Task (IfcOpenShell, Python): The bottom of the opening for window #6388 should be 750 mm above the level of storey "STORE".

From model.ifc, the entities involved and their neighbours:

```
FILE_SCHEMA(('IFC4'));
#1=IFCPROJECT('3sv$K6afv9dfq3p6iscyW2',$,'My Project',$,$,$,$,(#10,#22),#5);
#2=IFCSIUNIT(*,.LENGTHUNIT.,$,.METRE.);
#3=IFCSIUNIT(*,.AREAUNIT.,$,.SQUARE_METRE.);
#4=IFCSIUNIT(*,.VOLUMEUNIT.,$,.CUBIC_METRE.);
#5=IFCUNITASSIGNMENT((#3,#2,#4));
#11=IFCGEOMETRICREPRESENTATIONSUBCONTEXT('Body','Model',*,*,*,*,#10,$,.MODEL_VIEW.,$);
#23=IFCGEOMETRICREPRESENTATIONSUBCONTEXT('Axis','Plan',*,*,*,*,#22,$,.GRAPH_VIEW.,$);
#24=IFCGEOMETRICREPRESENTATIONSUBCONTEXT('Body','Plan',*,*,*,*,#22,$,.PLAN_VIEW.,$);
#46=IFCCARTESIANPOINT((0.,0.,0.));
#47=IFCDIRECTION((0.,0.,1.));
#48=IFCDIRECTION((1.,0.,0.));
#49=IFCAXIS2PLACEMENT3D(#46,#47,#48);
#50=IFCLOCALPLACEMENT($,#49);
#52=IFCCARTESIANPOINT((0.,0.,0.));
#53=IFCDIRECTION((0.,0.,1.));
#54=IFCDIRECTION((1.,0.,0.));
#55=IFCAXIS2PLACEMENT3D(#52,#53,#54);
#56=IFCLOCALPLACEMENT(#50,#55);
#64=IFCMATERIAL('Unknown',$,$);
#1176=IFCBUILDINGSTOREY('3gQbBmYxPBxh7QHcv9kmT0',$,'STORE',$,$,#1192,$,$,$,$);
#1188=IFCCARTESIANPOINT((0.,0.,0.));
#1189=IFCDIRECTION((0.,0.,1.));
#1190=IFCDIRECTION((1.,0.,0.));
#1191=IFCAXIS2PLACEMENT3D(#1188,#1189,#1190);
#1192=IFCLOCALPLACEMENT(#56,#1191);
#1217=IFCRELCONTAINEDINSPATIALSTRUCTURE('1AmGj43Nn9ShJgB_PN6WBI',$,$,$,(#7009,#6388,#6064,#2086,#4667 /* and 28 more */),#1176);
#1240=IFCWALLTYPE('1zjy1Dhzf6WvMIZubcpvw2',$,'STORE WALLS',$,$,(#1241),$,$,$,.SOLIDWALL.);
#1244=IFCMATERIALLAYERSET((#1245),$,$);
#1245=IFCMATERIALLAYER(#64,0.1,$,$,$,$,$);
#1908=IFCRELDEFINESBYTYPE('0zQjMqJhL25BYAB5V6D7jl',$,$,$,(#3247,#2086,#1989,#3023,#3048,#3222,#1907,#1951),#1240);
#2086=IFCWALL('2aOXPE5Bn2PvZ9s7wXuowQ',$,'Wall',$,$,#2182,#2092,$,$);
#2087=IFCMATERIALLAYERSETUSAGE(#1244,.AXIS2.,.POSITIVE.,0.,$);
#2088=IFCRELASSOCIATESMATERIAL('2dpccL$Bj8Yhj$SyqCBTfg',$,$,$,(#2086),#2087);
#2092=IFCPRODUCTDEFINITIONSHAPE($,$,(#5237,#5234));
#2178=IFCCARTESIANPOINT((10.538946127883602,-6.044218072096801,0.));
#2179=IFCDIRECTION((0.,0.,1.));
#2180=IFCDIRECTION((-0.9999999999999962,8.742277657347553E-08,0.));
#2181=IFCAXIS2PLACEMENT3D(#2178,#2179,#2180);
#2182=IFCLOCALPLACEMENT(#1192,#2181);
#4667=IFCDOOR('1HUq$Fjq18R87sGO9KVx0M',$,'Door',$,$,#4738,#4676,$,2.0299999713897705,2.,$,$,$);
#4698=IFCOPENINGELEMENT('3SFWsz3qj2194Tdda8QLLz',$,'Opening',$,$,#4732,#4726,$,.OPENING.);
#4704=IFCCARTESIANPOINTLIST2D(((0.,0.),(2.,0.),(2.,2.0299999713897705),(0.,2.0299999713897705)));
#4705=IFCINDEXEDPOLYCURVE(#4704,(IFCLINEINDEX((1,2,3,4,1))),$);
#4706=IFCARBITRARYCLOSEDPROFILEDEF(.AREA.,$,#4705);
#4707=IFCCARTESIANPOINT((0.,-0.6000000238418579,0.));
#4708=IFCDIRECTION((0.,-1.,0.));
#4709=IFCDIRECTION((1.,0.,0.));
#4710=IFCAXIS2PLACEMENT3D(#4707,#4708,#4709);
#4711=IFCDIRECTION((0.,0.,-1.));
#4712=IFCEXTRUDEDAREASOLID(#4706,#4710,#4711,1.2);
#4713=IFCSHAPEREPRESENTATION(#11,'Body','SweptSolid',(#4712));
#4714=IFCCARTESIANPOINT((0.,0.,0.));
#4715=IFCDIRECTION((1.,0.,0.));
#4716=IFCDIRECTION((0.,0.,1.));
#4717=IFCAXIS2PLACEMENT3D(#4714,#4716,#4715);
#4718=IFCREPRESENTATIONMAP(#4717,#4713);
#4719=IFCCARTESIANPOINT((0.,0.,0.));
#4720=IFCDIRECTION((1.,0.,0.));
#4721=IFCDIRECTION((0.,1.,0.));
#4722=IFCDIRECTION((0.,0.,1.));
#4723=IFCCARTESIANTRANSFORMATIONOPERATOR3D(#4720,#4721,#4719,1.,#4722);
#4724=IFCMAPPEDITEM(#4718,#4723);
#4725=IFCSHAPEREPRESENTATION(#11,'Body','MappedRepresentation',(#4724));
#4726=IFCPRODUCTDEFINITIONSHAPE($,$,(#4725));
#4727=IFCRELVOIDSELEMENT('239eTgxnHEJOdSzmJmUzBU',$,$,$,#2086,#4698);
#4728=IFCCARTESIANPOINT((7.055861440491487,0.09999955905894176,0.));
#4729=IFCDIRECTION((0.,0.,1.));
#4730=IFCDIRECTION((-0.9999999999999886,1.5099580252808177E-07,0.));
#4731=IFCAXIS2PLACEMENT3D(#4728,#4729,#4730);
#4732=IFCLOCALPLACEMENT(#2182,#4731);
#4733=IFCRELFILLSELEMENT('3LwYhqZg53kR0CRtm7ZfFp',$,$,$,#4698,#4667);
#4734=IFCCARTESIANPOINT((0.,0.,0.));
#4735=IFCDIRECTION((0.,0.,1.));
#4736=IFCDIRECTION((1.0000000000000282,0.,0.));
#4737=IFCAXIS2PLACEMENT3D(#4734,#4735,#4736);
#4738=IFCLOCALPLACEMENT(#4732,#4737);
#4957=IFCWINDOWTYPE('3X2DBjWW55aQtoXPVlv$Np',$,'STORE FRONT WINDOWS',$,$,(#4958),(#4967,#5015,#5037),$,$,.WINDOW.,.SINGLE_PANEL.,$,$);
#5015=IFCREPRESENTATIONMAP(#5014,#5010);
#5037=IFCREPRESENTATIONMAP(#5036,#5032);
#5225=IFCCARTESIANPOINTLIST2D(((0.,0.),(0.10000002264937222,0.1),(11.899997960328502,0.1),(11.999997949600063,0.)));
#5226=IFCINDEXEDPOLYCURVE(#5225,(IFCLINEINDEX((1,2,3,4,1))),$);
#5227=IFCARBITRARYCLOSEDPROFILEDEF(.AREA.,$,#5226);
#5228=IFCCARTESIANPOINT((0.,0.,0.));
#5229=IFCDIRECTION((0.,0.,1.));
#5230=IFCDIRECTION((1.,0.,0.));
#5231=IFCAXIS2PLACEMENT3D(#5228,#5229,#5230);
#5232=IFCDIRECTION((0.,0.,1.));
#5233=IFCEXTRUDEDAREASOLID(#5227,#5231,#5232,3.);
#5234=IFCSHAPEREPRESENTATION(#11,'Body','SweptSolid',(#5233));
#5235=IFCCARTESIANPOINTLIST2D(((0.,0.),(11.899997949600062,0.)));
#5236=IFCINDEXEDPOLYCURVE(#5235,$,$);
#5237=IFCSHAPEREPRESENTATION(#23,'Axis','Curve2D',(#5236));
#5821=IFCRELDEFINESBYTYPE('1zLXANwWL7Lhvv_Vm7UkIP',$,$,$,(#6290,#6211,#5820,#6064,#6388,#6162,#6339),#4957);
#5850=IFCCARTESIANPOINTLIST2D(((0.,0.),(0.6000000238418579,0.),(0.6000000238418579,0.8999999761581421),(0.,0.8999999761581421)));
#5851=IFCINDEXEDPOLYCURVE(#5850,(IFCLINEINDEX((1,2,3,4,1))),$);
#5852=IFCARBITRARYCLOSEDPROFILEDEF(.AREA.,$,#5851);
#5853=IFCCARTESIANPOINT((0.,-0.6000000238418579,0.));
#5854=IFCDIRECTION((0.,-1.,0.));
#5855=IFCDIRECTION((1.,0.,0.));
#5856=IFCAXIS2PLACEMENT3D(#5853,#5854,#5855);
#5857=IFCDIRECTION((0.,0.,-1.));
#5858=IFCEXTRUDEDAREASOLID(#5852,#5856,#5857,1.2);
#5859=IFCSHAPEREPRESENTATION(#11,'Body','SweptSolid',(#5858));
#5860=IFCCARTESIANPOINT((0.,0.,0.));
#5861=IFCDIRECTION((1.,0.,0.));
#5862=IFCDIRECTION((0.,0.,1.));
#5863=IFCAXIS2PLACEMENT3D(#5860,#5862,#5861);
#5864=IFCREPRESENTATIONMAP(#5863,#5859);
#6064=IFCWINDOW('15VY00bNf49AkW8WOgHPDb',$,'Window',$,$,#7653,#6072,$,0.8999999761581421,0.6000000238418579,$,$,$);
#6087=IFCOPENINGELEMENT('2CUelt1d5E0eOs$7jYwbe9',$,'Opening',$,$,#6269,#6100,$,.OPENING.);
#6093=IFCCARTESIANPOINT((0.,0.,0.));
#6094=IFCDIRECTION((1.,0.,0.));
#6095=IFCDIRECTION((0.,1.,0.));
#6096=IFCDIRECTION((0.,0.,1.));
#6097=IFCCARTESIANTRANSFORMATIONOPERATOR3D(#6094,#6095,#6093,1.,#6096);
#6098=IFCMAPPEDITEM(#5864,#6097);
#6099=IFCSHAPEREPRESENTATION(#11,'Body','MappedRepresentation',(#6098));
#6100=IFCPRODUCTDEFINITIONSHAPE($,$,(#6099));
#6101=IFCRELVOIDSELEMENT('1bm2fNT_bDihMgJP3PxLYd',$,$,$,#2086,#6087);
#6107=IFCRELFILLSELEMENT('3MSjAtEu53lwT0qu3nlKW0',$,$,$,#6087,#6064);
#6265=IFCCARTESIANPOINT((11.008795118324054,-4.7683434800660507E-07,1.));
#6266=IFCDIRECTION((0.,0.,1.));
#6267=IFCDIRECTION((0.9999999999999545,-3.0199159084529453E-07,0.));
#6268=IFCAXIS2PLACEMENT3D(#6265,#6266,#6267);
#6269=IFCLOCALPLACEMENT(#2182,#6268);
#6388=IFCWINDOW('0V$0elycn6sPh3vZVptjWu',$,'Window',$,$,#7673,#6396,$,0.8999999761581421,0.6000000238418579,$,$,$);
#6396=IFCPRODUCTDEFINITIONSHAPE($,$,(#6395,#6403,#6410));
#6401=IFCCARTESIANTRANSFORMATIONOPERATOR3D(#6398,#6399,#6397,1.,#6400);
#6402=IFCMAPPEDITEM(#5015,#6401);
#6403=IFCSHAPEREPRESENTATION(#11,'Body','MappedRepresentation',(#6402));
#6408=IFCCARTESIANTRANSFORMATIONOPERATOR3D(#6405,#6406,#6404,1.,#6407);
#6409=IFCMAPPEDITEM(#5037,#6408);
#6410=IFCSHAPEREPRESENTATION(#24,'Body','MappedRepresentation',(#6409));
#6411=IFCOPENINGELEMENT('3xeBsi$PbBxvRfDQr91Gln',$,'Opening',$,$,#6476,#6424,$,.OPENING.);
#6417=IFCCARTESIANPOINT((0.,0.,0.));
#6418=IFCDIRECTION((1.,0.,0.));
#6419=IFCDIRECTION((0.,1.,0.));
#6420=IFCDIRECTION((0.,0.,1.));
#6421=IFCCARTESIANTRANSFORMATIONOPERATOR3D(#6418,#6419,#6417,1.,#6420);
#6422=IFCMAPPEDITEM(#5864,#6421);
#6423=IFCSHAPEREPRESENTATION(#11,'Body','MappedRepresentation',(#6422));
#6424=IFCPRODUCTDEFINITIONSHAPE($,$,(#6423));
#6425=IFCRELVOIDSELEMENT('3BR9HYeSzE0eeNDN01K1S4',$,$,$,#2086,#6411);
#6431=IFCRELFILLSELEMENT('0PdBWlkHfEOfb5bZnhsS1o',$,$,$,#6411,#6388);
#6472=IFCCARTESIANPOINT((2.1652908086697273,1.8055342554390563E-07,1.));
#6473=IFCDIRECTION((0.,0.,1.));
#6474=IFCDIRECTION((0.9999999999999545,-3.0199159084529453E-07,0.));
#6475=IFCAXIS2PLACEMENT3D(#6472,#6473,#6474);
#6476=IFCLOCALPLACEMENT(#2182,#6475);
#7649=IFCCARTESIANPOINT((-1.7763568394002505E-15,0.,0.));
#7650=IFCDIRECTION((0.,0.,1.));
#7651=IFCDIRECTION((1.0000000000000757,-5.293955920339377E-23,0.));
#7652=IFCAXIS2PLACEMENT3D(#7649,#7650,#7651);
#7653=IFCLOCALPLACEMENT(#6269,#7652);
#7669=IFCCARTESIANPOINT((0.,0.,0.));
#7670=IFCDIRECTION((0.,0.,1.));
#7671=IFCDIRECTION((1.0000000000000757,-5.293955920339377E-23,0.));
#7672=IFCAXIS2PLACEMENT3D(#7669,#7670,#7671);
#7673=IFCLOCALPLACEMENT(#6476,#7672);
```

```python
import numpy as np
import ifcopenshell
import ifcopenshell.api.geometry
import ifcopenshell.geom
import ifcopenshell.util.element
import ifcopenshell.util.placement
import ifcopenshell.util.shape
import ifcopenshell.util.unit

model = ifcopenshell.open("model.ifc")
unit_scale = ifcopenshell.util.unit.calculate_unit_scale(model)

window = model.by_guid("0V$0elycn6sPh3vZVptjWu")
opening = window.FillsVoids[0].RelatingOpeningElement
storey = ifcopenshell.util.element.get_container(window, ifc_class="IfcBuildingStorey")
level = ifcopenshell.util.placement.get_local_placement(storey.ObjectPlacement)[2, 3]

# The opening's origin need not be at the sill, so measure its lowest point.
shape = ifcopenshell.geom.create_shape(ifcopenshell.geom.settings(), opening)
bottom = ifcopenshell.util.shape.get_shape_bottom_elevation(shape, shape.geometry) / unit_scale
dz = level + 0.75 - bottom

shift = np.array([0.0, 0.0, dz])
# The window is placed relative to its opening, so it follows when the opening moves.
matrix = ifcopenshell.util.placement.get_local_placement(opening.ObjectPlacement)
matrix[:3, 3] += shift
ifcopenshell.api.geometry.edit_object_placement(
    model, product=opening, matrix=matrix, is_si=False, should_transform_children=True
)

print(f"moved by {dz * unit_scale:+.3f} m")

model.write("model_edited.ifc")
```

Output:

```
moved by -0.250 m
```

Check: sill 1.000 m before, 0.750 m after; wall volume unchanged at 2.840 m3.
